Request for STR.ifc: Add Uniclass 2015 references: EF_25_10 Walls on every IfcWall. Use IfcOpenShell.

First a look at what the model holds.

```python
import ifcopenshell

model = ifcopenshell.open("STR.ifc")
print(model.schema)
print("classifications:", [c.Name for c in model.by_type("IfcClassification")])
for ifc_class in ("IfcDoor", "IfcRoof", "IfcStair", "IfcWall", "IfcWindow"):
    print(ifc_class, len(model.by_type(ifc_class)))
```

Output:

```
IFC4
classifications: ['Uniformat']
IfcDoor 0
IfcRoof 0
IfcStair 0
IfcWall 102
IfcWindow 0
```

```python
import ifcopenshell
import ifcopenshell.api.classification

model = ifcopenshell.open("STR.ifc")

system = ifcopenshell.api.classification.add_classification(model, classification="Uniclass 2015")

codes = {
    "IfcWall": ("EF_25_10", "Walls"),
}
for ifc_class, (code, name) in codes.items():
    products = model.by_type(ifc_class)
    ifcopenshell.api.classification.add_reference(
        model, products=products, classification=system, identification=code, name=name
    )
    print(code, len(products))

model.write("STR_v2.ifc")
```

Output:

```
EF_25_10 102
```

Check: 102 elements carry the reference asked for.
